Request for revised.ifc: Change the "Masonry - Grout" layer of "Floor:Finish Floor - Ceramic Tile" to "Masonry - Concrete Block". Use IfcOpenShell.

First a look at what the model holds.

```python
import ifcopenshell
import ifcopenshell.util.element

model = ifcopenshell.open("revised.ifc")
print(model.schema)
for layer_set in model.by_type("IfcMaterialLayerSet"):
    if layer_set.LayerSetName == "Floor:Finish Floor - Ceramic Tile":
        for layer in layer_set.MaterialLayers:
            print(layer.id(), layer.Material and layer.Material.Name, layer.LayerThickness, sep=" | ")
        print(len(ifcopenshell.util.element.get_elements_by_material(model, layer_set)), "elements and types use it")
print(sorted(m.Name for m in model.by_type("IfcMaterial") if m.Name)[:60])
```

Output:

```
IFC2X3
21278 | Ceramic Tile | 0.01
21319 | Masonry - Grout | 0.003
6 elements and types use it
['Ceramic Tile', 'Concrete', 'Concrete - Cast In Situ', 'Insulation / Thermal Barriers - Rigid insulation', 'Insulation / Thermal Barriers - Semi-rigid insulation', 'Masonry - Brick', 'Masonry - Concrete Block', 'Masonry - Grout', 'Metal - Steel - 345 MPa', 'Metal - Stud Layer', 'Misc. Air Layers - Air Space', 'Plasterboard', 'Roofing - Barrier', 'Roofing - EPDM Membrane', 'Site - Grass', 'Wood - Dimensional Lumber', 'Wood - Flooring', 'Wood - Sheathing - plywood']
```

```python
import ifcopenshell
import ifcopenshell.api.material

model = ifcopenshell.open("revised.ifc")

layer_set = next(s for s in model.by_type("IfcMaterialLayerSet") if s.LayerSetName == "Floor:Finish Floor - Ceramic Tile")
layer = next(l for l in layer_set.MaterialLayers if l.Material and l.Material.Name == "Masonry - Grout")
material = next(m for m in model.by_type("IfcMaterial") if m.Name == "Masonry - Concrete Block")

# Point this one layer at the other material; renaming the old one would change it everywhere.
ifcopenshell.api.material.edit_layer(model, layer=layer, attributes={}, material=material)

print([l.Material.Name if l.Material else None for l in layer_set.MaterialLayers])

model.write("revised_rev.ifc")
```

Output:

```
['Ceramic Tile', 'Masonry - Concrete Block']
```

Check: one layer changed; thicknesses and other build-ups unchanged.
